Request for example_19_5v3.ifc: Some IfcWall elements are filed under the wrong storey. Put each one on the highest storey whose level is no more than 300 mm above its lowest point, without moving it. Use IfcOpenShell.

First a look at what the model holds.

```python
import ifcopenshell
import ifcopenshell.util.element
import ifcopenshell.util.placement

model = ifcopenshell.open("example_19_5v3.ifc")
print(model.schema)
for storey in model.by_type("IfcBuildingStorey"):
    level = ifcopenshell.util.placement.get_storey_elevation(storey)
    count = sum(e.is_a("IfcWall") for e in ifcopenshell.util.element.get_contained(storey))
    print(storey.id(), storey.Name, round(level, 3), count, sep=" | ")
```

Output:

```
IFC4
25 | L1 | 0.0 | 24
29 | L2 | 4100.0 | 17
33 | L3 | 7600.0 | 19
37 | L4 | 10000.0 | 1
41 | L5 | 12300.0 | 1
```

```python
import ifcopenshell
import ifcopenshell.api.spatial
import ifcopenshell.geom
import ifcopenshell.util.element
import ifcopenshell.util.placement
import ifcopenshell.util.shape
import ifcopenshell.util.unit

model = ifcopenshell.open("example_19_5v3.ifc")
unit_scale = ifcopenshell.util.unit.calculate_unit_scale(model)
settings = ifcopenshell.geom.settings()

levels = sorted(
    ((ifcopenshell.util.placement.get_storey_elevation(s) * unit_scale, s) for s in model.by_type("IfcBuildingStorey")),
    key=lambda pair: pair[0],
)

for e in model.by_type("IfcWall"):
    current = e.ContainedInStructure[0].RelatingStructure if e.ContainedInStructure else None
    if current is None or not current.is_a("IfcBuildingStorey"):
        continue
    shape = ifcopenshell.geom.create_shape(settings, e)
    bottom = ifcopenshell.util.shape.get_shape_bottom_elevation(shape, shape.geometry)
    below = [s for level, s in levels if level <= bottom + 0.3]
    storey = below[-1] if below else levels[0][1]
    if storey != current:
        # assign_container keeps the world position.
        ifcopenshell.api.spatial.assign_container(model, products=[e], relating_structure=storey)
        print(e.id(), current.Name, "->", storey.Name)

model.write("example_19_5v3_rev.ifc")
```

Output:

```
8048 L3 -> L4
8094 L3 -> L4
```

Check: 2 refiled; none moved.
